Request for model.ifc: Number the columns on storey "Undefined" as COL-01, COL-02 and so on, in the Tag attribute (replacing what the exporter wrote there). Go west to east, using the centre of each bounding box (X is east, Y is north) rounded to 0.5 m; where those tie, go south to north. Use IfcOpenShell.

First a look at what the model holds.

```python
import ifcopenshell
import ifcopenshell.util.element
import ifcopenshell.util.placement

model = ifcopenshell.open("model.ifc")
print(model.schema)
storey = next(s for s in model.by_type("IfcBuildingStorey") if s.Name == "Undefined")
columns = [e for e in ifcopenshell.util.element.get_decomposition(storey) if e.is_a("IfcColumn")]
for e in sorted(columns, key=lambda e: e.id()):
    origin = ifcopenshell.util.placement.get_local_placement(e.ObjectPlacement)[:3, 3]
    print(e.id(), e.Tag, e.Name, origin.round(2) + 0.0, sep=" | ")
```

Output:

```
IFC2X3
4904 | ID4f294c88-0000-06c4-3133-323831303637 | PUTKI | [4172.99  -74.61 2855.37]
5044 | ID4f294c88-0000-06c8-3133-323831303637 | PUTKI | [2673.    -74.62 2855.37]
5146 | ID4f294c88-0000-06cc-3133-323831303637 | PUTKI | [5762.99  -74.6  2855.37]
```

```python
import ifcopenshell
import ifcopenshell.geom
import ifcopenshell.util.element
import ifcopenshell.util.shape

model = ifcopenshell.open("model.ifc")
settings = ifcopenshell.geom.settings()
settings.set("use-world-coords", True)


def centre(element):
    shape = ifcopenshell.geom.create_shape(settings, element)
    return ifcopenshell.util.shape.get_bbox_centroid(shape.geometry)


storey = next(s for s in model.by_type("IfcBuildingStorey") if s.Name == "Undefined")
columns = [e for e in ifcopenshell.util.element.get_decomposition(storey) if e.is_a("IfcColumn")]

# Insertion points can sit at a corner or the storey origin, so sort by the geometry (in metres).
centres = {e: centre(e) for e in columns}
columns.sort(key=lambda e: (round(centres[e][0] / 0.5), centres[e][1]))

for i, e in enumerate(columns, start=1):
    number = f"COL-{i:02d}"
    e.Tag = number
    print(e.id(), number)

model.write("model_edited.ifc")
```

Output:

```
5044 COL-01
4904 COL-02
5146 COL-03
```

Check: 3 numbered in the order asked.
